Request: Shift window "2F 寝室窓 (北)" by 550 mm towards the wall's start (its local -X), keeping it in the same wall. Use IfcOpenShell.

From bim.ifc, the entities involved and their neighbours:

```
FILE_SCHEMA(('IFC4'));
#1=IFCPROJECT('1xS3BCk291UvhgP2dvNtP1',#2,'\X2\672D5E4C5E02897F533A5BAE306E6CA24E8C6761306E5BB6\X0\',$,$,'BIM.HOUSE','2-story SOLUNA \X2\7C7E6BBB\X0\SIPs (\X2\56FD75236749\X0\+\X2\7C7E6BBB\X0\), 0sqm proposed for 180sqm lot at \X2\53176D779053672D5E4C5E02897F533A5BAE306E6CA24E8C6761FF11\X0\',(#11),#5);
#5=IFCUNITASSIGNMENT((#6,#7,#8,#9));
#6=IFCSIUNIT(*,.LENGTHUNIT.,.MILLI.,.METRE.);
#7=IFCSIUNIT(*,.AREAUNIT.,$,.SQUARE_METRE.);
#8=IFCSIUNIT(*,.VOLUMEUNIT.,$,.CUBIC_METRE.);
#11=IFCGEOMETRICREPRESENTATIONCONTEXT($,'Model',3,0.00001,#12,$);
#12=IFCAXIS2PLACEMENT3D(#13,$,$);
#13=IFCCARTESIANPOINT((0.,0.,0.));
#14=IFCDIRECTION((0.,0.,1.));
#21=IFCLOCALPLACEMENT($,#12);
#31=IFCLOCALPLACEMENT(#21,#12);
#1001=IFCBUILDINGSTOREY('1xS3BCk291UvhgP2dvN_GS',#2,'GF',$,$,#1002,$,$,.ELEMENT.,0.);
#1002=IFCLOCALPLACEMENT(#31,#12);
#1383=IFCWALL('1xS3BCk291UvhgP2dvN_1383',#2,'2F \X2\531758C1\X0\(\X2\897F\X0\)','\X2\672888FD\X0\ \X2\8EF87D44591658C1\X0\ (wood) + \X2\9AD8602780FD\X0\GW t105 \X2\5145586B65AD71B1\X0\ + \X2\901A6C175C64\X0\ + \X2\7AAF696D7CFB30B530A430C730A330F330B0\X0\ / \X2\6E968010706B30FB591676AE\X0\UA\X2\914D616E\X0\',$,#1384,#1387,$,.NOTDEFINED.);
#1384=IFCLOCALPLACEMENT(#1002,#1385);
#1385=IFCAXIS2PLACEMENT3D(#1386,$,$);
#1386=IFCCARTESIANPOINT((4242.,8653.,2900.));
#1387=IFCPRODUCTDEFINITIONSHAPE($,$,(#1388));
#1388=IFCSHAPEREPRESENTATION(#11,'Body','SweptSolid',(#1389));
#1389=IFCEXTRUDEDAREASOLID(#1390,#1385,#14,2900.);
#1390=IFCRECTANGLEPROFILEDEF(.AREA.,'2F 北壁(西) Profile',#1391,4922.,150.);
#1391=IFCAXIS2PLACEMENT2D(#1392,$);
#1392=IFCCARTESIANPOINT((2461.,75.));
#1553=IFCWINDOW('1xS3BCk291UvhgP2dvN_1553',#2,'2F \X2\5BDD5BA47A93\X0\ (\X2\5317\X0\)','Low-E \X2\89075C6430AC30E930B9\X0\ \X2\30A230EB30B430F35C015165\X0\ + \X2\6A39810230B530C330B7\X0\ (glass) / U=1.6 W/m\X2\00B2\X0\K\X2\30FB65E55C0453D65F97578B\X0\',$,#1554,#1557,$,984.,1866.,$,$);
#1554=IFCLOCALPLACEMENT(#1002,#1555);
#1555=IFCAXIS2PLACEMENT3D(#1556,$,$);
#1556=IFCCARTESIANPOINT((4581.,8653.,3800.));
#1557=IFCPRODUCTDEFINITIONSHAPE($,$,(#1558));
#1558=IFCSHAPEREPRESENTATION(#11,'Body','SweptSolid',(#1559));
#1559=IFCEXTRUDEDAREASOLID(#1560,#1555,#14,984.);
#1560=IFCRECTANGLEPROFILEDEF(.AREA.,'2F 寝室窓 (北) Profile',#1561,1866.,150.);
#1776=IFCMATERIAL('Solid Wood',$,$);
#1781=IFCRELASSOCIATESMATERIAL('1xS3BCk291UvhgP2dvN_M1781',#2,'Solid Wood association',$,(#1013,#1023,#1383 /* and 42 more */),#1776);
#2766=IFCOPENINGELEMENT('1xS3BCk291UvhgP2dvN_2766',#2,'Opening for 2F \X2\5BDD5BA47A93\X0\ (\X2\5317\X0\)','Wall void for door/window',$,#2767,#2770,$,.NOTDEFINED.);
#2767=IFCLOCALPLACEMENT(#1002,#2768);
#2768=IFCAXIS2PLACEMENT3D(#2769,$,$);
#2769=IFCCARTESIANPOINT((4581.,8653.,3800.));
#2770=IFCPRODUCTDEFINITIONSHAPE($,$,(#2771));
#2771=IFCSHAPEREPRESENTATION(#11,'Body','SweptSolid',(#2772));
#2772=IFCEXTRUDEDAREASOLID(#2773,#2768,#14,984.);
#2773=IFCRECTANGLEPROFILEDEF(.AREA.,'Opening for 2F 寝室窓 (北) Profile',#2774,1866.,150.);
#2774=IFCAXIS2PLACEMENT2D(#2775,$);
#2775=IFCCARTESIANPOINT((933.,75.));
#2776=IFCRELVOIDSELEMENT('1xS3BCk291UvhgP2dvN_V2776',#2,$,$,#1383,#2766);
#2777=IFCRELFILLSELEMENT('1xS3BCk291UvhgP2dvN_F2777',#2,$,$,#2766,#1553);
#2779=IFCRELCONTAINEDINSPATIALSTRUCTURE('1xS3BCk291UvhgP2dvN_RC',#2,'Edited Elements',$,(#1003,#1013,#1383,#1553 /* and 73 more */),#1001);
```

```python
import ifcopenshell
import ifcopenshell.api.geometry
import ifcopenshell.util.placement

model = ifcopenshell.open("bim.ifc")

window = model.by_id(1553)
opening = window.FillsVoids[0].RelatingOpeningElement
wall = opening.VoidsElements[0].RelatingBuildingElement

wall_matrix = ifcopenshell.util.placement.get_local_placement(wall.ObjectPlacement)
shift = wall_matrix[:3, 0] * -550.0
before = ifcopenshell.util.placement.get_local_placement(window.ObjectPlacement)[:3, 3].copy()

# The window is not placed relative to its opening, so move both.
for product in (opening, window):
    matrix = ifcopenshell.util.placement.get_local_placement(product.ObjectPlacement)
    matrix[:3, 3] += shift
    ifcopenshell.api.geometry.edit_object_placement(model, product=product, matrix=matrix, is_si=False)

after = ifcopenshell.util.placement.get_local_placement(window.ObjectPlacement)[:3, 3]
print("window moved by", (after - before).round(3) + 0.0)

model.write("bim-out.ifc")
```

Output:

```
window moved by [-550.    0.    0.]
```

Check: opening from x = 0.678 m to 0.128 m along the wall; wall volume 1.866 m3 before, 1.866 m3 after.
